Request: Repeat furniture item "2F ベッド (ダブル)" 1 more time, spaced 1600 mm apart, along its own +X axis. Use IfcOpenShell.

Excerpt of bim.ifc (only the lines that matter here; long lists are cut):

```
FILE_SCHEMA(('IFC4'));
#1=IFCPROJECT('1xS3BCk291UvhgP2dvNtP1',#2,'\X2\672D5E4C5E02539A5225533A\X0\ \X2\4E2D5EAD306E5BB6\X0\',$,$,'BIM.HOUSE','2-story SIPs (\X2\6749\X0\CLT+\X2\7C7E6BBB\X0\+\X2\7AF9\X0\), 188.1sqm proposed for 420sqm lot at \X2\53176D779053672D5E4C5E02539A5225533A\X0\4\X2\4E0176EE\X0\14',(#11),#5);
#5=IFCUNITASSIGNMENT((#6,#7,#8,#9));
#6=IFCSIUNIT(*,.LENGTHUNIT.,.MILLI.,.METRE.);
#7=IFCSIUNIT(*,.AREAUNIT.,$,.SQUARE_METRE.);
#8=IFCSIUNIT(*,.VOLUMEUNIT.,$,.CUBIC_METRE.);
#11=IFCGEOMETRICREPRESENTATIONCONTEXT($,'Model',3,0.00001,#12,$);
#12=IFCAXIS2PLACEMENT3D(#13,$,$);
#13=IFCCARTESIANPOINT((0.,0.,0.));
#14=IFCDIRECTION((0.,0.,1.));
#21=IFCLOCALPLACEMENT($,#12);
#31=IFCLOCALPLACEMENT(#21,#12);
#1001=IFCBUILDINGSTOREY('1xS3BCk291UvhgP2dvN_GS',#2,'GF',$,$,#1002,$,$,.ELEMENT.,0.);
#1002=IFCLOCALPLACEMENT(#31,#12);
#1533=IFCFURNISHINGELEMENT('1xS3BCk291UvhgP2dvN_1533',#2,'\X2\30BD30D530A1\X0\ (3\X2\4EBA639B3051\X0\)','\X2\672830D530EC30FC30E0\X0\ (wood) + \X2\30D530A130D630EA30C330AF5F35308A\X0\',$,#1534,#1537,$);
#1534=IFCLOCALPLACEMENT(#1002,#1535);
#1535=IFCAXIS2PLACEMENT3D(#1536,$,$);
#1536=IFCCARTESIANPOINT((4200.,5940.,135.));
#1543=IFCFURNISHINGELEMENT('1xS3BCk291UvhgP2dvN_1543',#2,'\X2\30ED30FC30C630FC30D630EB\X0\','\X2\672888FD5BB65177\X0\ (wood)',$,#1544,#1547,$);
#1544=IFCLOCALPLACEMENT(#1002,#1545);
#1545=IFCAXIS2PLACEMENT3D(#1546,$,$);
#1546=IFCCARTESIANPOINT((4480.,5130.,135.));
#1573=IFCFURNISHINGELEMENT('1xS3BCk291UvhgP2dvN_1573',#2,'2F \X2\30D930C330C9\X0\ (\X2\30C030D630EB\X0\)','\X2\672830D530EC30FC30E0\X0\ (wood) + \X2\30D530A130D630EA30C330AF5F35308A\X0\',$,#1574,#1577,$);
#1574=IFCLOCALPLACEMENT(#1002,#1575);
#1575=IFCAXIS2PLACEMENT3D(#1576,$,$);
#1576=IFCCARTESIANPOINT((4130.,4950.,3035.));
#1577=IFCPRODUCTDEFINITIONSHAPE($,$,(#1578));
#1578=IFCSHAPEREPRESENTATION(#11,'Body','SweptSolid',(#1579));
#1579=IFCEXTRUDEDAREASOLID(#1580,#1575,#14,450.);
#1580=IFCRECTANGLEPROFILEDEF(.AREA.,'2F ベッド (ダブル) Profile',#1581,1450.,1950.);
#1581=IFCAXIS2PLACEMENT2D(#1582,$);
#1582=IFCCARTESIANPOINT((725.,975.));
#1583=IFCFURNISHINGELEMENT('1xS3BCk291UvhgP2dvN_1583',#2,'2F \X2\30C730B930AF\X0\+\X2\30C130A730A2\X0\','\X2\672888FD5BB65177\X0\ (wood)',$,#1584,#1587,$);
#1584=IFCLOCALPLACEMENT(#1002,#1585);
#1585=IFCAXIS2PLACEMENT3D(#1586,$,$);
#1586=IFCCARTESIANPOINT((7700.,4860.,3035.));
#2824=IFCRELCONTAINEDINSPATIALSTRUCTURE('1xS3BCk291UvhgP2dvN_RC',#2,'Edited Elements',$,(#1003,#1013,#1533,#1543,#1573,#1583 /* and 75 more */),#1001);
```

```python
import ifcopenshell
import ifcopenshell.api.geometry
import ifcopenshell.api.root
import ifcopenshell.util.element
import ifcopenshell.util.placement
import ifcopenshell.util.unit

model = ifcopenshell.open("bim.ifc")
unit_scale = ifcopenshell.util.unit.calculate_unit_scale(model)


def reuse_history(source, copy):
    """copy_class also copies each property set's owner history, people and application; keep the originals."""
    for rel in copy.IsDefinedBy:
        if rel.is_a("IfcRelDefinesByProperties") and (history := rel.RelatingPropertyDefinition.OwnerHistory):
            rel.RelatingPropertyDefinition.OwnerHistory = source.OwnerHistory
            ifcopenshell.util.element.remove_deep2(model, history)


source = model.by_guid("1xS3BCk291UvhgP2dvN_1573")
base = ifcopenshell.util.placement.get_local_placement(source.ObjectPlacement)
step = base[:3, 0] * 1.6 / unit_scale

for i in range(1, 2):
    copy = ifcopenshell.api.root.copy_class(model, product=source)
    copy.Representation = ifcopenshell.util.element.copy_deep(
        model, source.Representation, exclude=["IfcGeometricRepresentationContext", "IfcRepresentationMap"]
    )
    reuse_history(source, copy)
    matrix = base.copy()
    matrix[:3, 3] += i * step
    print("added at", matrix[:3, 3].round(3) + 0.0)
    ifcopenshell.api.geometry.edit_object_placement(model, product=copy, matrix=matrix, is_si=False)

model.write("bim_edited.ifc")
```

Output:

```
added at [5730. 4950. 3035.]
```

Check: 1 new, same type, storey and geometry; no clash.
